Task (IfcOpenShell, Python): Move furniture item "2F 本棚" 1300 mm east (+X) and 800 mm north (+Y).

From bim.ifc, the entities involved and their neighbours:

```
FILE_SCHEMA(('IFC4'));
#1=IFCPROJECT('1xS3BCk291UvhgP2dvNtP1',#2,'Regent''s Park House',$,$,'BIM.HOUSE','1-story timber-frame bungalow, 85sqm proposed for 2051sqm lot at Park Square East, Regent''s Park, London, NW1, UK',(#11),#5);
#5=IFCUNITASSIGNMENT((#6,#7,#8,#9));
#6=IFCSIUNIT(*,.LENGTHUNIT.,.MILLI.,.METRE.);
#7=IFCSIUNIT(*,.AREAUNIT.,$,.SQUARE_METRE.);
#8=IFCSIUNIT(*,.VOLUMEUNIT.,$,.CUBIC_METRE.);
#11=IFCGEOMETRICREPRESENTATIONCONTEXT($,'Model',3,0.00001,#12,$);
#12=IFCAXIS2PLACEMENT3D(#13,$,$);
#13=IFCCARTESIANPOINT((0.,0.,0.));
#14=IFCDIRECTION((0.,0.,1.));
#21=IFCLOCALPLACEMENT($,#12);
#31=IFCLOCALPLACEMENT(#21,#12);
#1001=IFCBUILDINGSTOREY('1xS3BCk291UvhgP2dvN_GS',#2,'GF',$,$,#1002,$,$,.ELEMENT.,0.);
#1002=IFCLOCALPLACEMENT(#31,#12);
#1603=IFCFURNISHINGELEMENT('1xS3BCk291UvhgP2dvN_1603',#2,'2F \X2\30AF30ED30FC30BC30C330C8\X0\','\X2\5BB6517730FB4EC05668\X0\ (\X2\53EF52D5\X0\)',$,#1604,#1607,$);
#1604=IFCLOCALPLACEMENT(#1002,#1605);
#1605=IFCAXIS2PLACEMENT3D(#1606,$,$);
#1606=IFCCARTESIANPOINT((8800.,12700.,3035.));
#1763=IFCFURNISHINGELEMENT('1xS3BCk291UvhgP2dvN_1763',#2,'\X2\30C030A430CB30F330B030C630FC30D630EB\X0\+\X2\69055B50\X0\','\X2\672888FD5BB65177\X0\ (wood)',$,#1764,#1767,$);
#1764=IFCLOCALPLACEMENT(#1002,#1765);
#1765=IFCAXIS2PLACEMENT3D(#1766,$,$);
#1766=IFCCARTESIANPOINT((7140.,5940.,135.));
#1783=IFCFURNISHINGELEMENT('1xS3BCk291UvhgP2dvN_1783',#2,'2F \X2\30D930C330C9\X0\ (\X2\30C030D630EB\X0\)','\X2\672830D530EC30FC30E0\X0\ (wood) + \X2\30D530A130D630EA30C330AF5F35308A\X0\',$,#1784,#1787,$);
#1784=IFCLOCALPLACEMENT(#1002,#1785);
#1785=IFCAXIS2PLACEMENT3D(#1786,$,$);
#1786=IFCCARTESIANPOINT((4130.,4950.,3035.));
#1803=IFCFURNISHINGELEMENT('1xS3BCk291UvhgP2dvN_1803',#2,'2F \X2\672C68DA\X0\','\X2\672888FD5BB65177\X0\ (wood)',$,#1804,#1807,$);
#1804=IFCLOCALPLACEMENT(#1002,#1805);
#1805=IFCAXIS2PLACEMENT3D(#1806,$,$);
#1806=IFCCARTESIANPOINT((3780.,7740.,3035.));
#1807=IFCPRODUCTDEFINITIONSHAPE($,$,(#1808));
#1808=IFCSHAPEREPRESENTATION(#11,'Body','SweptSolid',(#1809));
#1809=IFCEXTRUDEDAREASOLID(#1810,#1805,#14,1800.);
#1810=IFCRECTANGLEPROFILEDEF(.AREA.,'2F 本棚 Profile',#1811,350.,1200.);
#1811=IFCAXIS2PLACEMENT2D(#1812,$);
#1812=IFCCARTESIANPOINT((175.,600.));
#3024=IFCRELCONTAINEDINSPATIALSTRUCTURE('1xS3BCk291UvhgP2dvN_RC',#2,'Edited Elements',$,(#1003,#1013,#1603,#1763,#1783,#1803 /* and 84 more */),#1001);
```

```python
import ifcopenshell
import ifcopenshell.api.geometry
import ifcopenshell.util.placement
import ifcopenshell.util.unit

model = ifcopenshell.open("bim.ifc")
unit_scale = ifcopenshell.util.unit.calculate_unit_scale(model)

item = model.by_guid("1xS3BCk291UvhgP2dvN_1803")
matrix = ifcopenshell.util.placement.get_local_placement(item.ObjectPlacement)
matrix[0, 3] += 1.3 / unit_scale
matrix[1, 3] += 0.8 / unit_scale
ifcopenshell.api.geometry.edit_object_placement(model, product=item, matrix=matrix, is_si=False)

print(ifcopenshell.util.placement.get_local_placement(item.ObjectPlacement).round(3) + 0.0)

model.write("bim_updated.ifc")
```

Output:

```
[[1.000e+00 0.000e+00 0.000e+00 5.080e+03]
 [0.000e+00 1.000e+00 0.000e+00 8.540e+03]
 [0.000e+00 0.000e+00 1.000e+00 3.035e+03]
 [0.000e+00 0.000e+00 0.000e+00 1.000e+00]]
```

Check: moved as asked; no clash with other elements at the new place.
